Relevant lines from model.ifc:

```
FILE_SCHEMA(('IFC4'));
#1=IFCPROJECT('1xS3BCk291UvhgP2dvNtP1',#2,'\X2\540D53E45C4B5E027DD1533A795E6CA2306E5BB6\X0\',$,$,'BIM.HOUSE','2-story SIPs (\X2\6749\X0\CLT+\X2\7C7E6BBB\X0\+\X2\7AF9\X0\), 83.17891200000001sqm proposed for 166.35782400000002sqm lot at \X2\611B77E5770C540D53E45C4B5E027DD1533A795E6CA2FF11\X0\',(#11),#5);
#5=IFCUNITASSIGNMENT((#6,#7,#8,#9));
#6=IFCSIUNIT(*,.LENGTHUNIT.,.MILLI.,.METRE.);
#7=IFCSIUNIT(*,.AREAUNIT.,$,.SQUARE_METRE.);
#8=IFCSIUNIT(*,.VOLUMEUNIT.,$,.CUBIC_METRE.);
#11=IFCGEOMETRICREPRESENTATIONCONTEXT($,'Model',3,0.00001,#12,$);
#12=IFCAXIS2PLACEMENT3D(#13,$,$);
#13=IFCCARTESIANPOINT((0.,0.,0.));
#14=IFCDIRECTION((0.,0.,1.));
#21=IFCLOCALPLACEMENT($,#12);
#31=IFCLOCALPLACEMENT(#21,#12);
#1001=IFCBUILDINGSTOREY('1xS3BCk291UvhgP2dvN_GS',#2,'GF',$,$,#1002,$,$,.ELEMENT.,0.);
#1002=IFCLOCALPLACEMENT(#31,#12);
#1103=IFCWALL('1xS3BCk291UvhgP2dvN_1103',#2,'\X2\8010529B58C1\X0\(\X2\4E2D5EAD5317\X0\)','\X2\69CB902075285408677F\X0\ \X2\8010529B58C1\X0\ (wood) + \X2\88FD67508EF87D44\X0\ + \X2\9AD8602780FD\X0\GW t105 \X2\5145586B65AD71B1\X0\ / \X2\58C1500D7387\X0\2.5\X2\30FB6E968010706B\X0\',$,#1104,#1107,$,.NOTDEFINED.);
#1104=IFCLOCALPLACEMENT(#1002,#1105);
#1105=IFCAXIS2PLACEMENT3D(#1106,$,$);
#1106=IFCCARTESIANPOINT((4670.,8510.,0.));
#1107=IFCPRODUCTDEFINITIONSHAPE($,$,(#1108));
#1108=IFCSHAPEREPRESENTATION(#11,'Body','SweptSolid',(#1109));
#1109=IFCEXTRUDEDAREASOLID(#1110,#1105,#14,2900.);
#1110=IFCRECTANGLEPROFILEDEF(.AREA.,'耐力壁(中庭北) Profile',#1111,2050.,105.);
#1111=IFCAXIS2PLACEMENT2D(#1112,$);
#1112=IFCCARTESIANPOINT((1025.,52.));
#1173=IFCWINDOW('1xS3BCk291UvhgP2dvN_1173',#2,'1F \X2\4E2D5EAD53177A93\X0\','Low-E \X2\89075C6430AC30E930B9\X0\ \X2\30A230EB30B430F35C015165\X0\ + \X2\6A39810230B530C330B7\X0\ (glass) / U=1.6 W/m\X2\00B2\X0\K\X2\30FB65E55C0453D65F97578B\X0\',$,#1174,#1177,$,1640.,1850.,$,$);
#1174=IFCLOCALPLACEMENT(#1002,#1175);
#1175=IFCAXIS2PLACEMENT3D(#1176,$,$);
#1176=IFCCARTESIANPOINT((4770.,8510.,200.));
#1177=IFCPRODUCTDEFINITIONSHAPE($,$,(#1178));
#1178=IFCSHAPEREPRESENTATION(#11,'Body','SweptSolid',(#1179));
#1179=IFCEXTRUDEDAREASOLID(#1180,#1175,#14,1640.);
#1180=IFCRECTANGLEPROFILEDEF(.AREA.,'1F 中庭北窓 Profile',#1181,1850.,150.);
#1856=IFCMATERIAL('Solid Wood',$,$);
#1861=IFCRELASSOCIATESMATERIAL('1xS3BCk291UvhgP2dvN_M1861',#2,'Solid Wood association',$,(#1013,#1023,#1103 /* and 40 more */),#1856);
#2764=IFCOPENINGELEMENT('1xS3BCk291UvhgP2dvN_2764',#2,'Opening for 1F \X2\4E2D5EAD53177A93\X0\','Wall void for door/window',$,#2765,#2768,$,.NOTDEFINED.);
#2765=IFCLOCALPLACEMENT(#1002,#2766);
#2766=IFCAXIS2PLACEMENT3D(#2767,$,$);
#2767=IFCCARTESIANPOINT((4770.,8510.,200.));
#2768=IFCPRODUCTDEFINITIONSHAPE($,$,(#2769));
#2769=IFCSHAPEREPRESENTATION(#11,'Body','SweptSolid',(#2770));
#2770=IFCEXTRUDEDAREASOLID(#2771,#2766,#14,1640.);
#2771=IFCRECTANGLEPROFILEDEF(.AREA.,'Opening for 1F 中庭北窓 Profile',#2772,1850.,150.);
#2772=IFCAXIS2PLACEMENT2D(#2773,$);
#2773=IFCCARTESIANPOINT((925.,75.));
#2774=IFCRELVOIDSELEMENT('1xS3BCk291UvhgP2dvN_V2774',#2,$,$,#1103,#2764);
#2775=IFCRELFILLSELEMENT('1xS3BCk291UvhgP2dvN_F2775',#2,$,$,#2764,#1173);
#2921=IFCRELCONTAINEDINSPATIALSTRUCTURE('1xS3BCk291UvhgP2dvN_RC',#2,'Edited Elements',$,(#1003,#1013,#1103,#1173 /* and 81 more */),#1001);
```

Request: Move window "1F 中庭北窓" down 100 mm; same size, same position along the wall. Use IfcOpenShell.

```python
import numpy as np
import ifcopenshell
import ifcopenshell.api.geometry
import ifcopenshell.util.placement
import ifcopenshell.util.unit

model = ifcopenshell.open("model.ifc")
unit_scale = ifcopenshell.util.unit.calculate_unit_scale(model)

window = model.by_id(1173)
opening = window.FillsVoids[0].RelatingOpeningElement
dz = -0.1 / unit_scale

shift = np.array([0.0, 0.0, dz])
# The window is not placed relative to its opening, so move both.
for product in (opening, window):
    matrix = ifcopenshell.util.placement.get_local_placement(product.ObjectPlacement)
    matrix[:3, 3] += shift
    ifcopenshell.api.geometry.edit_object_placement(model, product=product, matrix=matrix, is_si=False)

print(f"moved by {dz * unit_scale:+.3f} m")

model.write("model_updated.ifc")
```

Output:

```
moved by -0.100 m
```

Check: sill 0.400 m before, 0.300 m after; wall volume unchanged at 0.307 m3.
